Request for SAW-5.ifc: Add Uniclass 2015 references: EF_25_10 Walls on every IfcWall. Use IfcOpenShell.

First a look at what the model holds.

```python
import ifcopenshell

model = ifcopenshell.open("SAW-5.ifc")
print(model.schema)
print("classifications:", [c.Name for c in model.by_type("IfcClassification")])
for ifc_class in ("IfcDoor", "IfcRoof", "IfcStair", "IfcWall", "IfcWindow"):
    print(ifc_class, len(model.by_type(ifc_class)))
```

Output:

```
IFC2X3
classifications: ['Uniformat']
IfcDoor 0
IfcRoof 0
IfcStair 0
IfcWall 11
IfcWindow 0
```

```python
import ifcopenshell
import ifcopenshell.api.classification

model = ifcopenshell.open("SAW-5.ifc")

# IFC2X3 requires Source and Edition and has no link from the project to the system.
system = model.create_entity("IfcClassification", Source="NBS", Edition="2015", Name="Uniclass 2015")

codes = {
    "IfcWall": ("EF_25_10", "Walls"),
}
for ifc_class, (code, name) in codes.items():
    products = model.by_type(ifc_class)
    ifcopenshell.api.classification.add_reference(
        model, products=products, classification=system, identification=code, name=name
    )
    print(code, len(products))

model.write("SAW-5_rev.ifc")
```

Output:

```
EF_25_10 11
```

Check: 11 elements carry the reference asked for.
